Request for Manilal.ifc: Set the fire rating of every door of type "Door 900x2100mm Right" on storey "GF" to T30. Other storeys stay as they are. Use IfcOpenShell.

First a look at what the model holds.

```python
import ifcopenshell
import ifcopenshell.util.element

model = ifcopenshell.open("Manilal.ifc")
print(model.schema)
storey = next(s for s in model.by_type("IfcBuildingStorey") if s.Name == "GF")
doors = [e for e in ifcopenshell.util.element.get_decomposition(storey) if e.is_a("IfcDoor")]
seen = {}
for e in doors:
    element_type = ifcopenshell.util.element.get_type(e)
    key = (element_type.Name if element_type != e and element_type else None, ifcopenshell.util.element.get_pset(e, "Pset_DoorCommon", "FireRating"))
    seen[key] = seen.get(key, 0) + 1
for (name, value), count in sorted(seen.items(), key=str):
    print(count, "x", name, "|", value)
```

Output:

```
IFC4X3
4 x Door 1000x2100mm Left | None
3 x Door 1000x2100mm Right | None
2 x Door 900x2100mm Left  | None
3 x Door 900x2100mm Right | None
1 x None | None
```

```python
import ifcopenshell
import ifcopenshell.api.pset
import ifcopenshell.util.element

model = ifcopenshell.open("Manilal.ifc")

storey = next(s for s in model.by_type("IfcBuildingStorey") if s.Name == "GF")
doors = [e for e in ifcopenshell.util.element.get_decomposition(storey) if e.is_a("IfcDoor")]

count = 0
for e in doors:
    element_type = ifcopenshell.util.element.get_type(e)
    if element_type in (None, e) or element_type.Name != "Door 900x2100mm Right":
        continue
    # add_pset returns the element's existing set when there is one.
    pset = ifcopenshell.api.pset.add_pset(model, product=e, name="Pset_DoorCommon")
    ifcopenshell.api.pset.edit_pset(model, pset=pset, properties={"FireRating": "T30"})
    count += 1

print(count, "doors updated")

model.write("Manilal_v2.ifc")
```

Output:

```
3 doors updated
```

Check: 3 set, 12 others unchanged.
